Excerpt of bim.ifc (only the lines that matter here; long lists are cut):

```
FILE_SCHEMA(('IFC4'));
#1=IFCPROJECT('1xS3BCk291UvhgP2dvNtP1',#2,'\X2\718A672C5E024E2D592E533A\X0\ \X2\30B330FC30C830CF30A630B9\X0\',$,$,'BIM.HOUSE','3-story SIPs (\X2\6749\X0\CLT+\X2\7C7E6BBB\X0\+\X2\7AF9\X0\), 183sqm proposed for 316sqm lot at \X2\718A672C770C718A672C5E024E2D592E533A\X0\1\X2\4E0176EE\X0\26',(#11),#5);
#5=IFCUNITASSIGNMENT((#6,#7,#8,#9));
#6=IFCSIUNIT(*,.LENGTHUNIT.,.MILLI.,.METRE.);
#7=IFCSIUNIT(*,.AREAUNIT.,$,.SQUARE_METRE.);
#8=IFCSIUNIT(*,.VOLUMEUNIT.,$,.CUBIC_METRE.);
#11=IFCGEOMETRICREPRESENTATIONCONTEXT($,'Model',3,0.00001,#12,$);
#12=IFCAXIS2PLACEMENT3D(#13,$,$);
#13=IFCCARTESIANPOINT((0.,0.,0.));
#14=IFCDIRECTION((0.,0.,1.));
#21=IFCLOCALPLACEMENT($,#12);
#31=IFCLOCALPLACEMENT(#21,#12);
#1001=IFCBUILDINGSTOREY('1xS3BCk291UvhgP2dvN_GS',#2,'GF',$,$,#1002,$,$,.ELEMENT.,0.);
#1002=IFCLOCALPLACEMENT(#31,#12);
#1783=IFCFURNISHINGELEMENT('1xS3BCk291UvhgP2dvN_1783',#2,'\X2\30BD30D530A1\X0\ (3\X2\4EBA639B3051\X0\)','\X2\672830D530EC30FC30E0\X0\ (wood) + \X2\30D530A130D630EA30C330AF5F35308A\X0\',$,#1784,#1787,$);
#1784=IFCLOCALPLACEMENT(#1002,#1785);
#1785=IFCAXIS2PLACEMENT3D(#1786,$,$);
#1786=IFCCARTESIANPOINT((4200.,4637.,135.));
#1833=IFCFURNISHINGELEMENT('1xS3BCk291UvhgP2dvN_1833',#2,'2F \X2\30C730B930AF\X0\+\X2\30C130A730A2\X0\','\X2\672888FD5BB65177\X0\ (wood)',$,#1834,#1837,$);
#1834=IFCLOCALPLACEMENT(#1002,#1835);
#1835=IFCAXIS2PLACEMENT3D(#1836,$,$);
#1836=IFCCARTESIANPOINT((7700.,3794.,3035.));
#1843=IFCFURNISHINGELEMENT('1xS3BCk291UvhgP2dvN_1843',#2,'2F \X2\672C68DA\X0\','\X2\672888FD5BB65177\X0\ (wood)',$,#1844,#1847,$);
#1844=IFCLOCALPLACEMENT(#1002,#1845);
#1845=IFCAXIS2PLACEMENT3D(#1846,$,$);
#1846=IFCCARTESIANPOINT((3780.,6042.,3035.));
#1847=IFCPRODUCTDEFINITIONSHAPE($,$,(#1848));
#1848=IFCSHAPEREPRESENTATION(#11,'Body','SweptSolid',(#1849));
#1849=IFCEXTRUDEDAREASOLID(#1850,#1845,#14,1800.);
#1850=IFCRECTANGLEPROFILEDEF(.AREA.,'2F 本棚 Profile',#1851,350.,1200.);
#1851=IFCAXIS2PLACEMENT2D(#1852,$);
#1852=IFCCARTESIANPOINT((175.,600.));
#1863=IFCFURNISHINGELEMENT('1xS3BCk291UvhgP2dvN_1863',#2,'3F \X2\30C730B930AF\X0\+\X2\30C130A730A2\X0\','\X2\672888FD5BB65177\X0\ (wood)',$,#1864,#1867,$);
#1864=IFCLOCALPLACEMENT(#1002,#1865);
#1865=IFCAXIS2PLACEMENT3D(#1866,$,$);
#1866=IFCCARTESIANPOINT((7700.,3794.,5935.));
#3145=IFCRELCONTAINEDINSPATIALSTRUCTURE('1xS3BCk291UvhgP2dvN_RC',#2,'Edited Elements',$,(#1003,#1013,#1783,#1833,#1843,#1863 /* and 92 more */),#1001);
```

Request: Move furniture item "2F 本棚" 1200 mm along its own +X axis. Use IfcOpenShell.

```python
import ifcopenshell
import ifcopenshell.api.geometry
import ifcopenshell.util.placement

model = ifcopenshell.open("bim.ifc")

item = model.by_id(1843)
matrix = ifcopenshell.util.placement.get_local_placement(item.ObjectPlacement)
matrix[:3, 3] += matrix[:3, 0] * 1200.0
ifcopenshell.api.geometry.edit_object_placement(model, product=item, matrix=matrix, is_si=False)

print(ifcopenshell.util.placement.get_local_placement(item.ObjectPlacement).round(3) + 0.0)

model.write("bim_updated.ifc")
```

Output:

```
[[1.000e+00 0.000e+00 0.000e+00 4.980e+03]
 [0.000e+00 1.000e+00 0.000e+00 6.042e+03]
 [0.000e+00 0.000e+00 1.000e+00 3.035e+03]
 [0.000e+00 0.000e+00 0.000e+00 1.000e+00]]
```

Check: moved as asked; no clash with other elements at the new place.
